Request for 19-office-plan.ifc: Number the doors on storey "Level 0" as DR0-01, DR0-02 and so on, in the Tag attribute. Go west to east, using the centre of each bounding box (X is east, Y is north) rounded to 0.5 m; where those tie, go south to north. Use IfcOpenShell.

First a look at what the model holds.

```python
import ifcopenshell
import ifcopenshell.util.element
import ifcopenshell.util.placement

model = ifcopenshell.open("19-office-plan.ifc")
print(model.schema)
storey = next(s for s in model.by_type("IfcBuildingStorey") if s.Name == "Level 0")
doors = [e for e in ifcopenshell.util.element.get_decomposition(storey) if e.is_a("IfcDoor")]
for e in sorted(doors, key=lambda e: e.id()):
    origin = ifcopenshell.util.placement.get_local_placement(e.ObjectPlacement)[:3, 3]
    print(e.id(), e.Tag, e.Name, origin.round(2) + 0.0, sep=" | ")
```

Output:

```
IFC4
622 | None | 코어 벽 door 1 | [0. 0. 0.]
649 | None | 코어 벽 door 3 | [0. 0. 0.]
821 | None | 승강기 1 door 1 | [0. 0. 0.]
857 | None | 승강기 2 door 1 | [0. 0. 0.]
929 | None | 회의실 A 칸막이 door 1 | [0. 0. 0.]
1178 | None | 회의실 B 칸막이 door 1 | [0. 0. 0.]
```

```python
import ifcopenshell
import ifcopenshell.geom
import ifcopenshell.util.element
import ifcopenshell.util.shape

model = ifcopenshell.open("19-office-plan.ifc")
settings = ifcopenshell.geom.settings()
settings.set("use-world-coords", True)


def centre(element):
    shape = ifcopenshell.geom.create_shape(settings, element)
    return ifcopenshell.util.shape.get_bbox_centroid(shape.geometry)


storey = next(s for s in model.by_type("IfcBuildingStorey") if s.Name == "Level 0")
doors = [e for e in ifcopenshell.util.element.get_decomposition(storey) if e.is_a("IfcDoor")]

# Insertion points can sit at a corner or the storey origin, so sort by the geometry (in metres).
centres = {e: centre(e) for e in doors}
doors.sort(key=lambda e: (round(centres[e][0] / 0.5), centres[e][1]))

for i, e in enumerate(doors, start=1):
    number = f"DR0-{i:02d}"
    e.Tag = number
    print(e.id(), number)

model.write("19-office-plan-out.ifc")
```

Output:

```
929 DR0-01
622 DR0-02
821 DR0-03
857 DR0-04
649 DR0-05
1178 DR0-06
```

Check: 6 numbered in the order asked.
